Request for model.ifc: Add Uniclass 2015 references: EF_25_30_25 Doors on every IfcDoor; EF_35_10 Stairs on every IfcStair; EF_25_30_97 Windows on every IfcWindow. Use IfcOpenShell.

First a look at what the model holds.

```python
import ifcopenshell

model = ifcopenshell.open("model.ifc")
print(model.schema)
print("classifications:", [c.Name for c in model.by_type("IfcClassification")])
for ifc_class in ("IfcDoor", "IfcRoof", "IfcStair", "IfcWall", "IfcWindow"):
    print(ifc_class, len(model.by_type(ifc_class)))
```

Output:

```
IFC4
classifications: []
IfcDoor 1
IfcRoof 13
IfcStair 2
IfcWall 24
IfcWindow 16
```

```python
import ifcopenshell
import ifcopenshell.api.classification

model = ifcopenshell.open("model.ifc")

system = ifcopenshell.api.classification.add_classification(model, classification="Uniclass 2015")

codes = {
    "IfcDoor": ("EF_25_30_25", "Doors"),
    "IfcStair": ("EF_35_10", "Stairs"),
    "IfcWindow": ("EF_25_30_97", "Windows"),
}
for ifc_class, (code, name) in codes.items():
    products = model.by_type(ifc_class)
    ifcopenshell.api.classification.add_reference(
        model, products=products, classification=system, identification=code, name=name
    )
    print(code, len(products))

model.write("model_updated.ifc")
```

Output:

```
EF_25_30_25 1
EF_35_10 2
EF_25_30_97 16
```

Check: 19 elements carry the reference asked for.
